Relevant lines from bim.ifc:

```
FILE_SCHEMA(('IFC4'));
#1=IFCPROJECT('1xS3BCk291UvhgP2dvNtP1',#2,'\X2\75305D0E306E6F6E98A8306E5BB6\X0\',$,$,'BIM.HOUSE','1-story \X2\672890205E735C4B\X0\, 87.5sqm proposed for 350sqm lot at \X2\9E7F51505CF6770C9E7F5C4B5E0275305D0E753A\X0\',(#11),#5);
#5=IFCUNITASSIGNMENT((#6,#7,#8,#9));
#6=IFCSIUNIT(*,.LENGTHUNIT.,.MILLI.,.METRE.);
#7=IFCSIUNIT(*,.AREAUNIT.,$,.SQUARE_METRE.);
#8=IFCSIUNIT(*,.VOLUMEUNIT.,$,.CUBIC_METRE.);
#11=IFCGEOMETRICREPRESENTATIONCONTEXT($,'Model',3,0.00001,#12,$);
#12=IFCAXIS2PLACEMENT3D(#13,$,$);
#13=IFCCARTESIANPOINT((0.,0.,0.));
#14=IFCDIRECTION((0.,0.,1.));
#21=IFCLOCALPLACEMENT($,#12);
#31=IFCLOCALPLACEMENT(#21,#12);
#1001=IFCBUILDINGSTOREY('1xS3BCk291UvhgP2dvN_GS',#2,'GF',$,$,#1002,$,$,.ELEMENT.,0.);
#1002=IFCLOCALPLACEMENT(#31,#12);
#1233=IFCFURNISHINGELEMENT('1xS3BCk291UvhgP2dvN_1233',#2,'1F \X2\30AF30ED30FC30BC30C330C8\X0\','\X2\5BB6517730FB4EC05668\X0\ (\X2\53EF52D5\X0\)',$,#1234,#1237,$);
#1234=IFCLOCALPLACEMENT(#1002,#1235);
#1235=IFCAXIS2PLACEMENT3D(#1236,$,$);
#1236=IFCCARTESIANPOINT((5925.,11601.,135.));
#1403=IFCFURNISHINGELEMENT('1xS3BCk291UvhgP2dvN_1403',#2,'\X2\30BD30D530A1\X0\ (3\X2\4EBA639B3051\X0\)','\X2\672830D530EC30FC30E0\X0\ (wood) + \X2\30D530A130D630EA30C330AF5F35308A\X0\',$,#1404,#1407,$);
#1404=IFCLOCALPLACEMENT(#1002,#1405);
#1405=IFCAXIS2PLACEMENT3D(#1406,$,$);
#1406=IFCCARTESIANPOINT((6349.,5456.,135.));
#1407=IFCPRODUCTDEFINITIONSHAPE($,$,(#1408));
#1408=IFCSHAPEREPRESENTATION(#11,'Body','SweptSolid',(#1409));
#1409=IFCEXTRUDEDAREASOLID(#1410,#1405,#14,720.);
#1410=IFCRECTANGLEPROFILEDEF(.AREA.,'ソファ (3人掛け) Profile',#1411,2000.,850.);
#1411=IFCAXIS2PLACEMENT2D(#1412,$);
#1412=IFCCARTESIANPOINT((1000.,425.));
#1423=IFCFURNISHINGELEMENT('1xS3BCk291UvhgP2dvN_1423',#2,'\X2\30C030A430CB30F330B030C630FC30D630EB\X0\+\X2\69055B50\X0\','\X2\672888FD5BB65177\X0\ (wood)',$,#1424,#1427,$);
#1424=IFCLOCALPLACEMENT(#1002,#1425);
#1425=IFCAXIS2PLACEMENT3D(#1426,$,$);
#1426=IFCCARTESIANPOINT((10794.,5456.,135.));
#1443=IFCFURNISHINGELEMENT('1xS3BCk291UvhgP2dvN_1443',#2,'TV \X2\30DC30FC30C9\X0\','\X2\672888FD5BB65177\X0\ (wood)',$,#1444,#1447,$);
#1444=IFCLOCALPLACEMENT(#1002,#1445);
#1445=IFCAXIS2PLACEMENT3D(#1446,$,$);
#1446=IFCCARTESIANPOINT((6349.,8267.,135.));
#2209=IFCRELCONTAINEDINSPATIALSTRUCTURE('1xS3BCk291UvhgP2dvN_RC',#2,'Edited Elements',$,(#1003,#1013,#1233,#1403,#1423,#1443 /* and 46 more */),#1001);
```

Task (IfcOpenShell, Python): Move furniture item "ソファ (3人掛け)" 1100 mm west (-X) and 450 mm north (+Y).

```python
import ifcopenshell
import ifcopenshell.api.geometry
import ifcopenshell.util.placement
import ifcopenshell.util.unit

model = ifcopenshell.open("bim.ifc")
unit_scale = ifcopenshell.util.unit.calculate_unit_scale(model)

item = model.by_id(1403)
matrix = ifcopenshell.util.placement.get_local_placement(item.ObjectPlacement)
matrix[0, 3] -= 1.1 / unit_scale
matrix[1, 3] += 0.45 / unit_scale
ifcopenshell.api.geometry.edit_object_placement(model, product=item, matrix=matrix, is_si=False)

print(ifcopenshell.util.placement.get_local_placement(item.ObjectPlacement).round(3) + 0.0)

model.write("bim-out.ifc")
```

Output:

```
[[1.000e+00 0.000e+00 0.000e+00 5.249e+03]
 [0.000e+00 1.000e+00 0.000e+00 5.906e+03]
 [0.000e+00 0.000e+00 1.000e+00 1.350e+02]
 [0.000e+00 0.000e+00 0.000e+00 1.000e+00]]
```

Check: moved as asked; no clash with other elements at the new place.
